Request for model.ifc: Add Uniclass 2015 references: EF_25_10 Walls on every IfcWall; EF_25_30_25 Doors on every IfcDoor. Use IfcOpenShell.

First a look at what the model holds.

```python
import ifcopenshell

model = ifcopenshell.open("model.ifc")
print(model.schema)
print("classifications:", [c.Name for c in model.by_type("IfcClassification")])
for ifc_class in ("IfcDoor", "IfcRoof", "IfcStair", "IfcWall", "IfcWindow"):
    print(ifc_class, len(model.by_type(ifc_class)))
```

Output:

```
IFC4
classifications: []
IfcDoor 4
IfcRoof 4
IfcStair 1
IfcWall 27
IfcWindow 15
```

```python
import ifcopenshell
import ifcopenshell.api.classification

model = ifcopenshell.open("model.ifc")

system = ifcopenshell.api.classification.add_classification(model, classification="Uniclass 2015")

codes = {
    "IfcWall": ("EF_25_10", "Walls"),
    "IfcDoor": ("EF_25_30_25", "Doors"),
}
for ifc_class, (code, name) in codes.items():
    products = model.by_type(ifc_class)
    ifcopenshell.api.classification.add_reference(
        model, products=products, classification=system, identification=code, name=name
    )
    print(code, len(products))

model.write("model_v2.ifc")
```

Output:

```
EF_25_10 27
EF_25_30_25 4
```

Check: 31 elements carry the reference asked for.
